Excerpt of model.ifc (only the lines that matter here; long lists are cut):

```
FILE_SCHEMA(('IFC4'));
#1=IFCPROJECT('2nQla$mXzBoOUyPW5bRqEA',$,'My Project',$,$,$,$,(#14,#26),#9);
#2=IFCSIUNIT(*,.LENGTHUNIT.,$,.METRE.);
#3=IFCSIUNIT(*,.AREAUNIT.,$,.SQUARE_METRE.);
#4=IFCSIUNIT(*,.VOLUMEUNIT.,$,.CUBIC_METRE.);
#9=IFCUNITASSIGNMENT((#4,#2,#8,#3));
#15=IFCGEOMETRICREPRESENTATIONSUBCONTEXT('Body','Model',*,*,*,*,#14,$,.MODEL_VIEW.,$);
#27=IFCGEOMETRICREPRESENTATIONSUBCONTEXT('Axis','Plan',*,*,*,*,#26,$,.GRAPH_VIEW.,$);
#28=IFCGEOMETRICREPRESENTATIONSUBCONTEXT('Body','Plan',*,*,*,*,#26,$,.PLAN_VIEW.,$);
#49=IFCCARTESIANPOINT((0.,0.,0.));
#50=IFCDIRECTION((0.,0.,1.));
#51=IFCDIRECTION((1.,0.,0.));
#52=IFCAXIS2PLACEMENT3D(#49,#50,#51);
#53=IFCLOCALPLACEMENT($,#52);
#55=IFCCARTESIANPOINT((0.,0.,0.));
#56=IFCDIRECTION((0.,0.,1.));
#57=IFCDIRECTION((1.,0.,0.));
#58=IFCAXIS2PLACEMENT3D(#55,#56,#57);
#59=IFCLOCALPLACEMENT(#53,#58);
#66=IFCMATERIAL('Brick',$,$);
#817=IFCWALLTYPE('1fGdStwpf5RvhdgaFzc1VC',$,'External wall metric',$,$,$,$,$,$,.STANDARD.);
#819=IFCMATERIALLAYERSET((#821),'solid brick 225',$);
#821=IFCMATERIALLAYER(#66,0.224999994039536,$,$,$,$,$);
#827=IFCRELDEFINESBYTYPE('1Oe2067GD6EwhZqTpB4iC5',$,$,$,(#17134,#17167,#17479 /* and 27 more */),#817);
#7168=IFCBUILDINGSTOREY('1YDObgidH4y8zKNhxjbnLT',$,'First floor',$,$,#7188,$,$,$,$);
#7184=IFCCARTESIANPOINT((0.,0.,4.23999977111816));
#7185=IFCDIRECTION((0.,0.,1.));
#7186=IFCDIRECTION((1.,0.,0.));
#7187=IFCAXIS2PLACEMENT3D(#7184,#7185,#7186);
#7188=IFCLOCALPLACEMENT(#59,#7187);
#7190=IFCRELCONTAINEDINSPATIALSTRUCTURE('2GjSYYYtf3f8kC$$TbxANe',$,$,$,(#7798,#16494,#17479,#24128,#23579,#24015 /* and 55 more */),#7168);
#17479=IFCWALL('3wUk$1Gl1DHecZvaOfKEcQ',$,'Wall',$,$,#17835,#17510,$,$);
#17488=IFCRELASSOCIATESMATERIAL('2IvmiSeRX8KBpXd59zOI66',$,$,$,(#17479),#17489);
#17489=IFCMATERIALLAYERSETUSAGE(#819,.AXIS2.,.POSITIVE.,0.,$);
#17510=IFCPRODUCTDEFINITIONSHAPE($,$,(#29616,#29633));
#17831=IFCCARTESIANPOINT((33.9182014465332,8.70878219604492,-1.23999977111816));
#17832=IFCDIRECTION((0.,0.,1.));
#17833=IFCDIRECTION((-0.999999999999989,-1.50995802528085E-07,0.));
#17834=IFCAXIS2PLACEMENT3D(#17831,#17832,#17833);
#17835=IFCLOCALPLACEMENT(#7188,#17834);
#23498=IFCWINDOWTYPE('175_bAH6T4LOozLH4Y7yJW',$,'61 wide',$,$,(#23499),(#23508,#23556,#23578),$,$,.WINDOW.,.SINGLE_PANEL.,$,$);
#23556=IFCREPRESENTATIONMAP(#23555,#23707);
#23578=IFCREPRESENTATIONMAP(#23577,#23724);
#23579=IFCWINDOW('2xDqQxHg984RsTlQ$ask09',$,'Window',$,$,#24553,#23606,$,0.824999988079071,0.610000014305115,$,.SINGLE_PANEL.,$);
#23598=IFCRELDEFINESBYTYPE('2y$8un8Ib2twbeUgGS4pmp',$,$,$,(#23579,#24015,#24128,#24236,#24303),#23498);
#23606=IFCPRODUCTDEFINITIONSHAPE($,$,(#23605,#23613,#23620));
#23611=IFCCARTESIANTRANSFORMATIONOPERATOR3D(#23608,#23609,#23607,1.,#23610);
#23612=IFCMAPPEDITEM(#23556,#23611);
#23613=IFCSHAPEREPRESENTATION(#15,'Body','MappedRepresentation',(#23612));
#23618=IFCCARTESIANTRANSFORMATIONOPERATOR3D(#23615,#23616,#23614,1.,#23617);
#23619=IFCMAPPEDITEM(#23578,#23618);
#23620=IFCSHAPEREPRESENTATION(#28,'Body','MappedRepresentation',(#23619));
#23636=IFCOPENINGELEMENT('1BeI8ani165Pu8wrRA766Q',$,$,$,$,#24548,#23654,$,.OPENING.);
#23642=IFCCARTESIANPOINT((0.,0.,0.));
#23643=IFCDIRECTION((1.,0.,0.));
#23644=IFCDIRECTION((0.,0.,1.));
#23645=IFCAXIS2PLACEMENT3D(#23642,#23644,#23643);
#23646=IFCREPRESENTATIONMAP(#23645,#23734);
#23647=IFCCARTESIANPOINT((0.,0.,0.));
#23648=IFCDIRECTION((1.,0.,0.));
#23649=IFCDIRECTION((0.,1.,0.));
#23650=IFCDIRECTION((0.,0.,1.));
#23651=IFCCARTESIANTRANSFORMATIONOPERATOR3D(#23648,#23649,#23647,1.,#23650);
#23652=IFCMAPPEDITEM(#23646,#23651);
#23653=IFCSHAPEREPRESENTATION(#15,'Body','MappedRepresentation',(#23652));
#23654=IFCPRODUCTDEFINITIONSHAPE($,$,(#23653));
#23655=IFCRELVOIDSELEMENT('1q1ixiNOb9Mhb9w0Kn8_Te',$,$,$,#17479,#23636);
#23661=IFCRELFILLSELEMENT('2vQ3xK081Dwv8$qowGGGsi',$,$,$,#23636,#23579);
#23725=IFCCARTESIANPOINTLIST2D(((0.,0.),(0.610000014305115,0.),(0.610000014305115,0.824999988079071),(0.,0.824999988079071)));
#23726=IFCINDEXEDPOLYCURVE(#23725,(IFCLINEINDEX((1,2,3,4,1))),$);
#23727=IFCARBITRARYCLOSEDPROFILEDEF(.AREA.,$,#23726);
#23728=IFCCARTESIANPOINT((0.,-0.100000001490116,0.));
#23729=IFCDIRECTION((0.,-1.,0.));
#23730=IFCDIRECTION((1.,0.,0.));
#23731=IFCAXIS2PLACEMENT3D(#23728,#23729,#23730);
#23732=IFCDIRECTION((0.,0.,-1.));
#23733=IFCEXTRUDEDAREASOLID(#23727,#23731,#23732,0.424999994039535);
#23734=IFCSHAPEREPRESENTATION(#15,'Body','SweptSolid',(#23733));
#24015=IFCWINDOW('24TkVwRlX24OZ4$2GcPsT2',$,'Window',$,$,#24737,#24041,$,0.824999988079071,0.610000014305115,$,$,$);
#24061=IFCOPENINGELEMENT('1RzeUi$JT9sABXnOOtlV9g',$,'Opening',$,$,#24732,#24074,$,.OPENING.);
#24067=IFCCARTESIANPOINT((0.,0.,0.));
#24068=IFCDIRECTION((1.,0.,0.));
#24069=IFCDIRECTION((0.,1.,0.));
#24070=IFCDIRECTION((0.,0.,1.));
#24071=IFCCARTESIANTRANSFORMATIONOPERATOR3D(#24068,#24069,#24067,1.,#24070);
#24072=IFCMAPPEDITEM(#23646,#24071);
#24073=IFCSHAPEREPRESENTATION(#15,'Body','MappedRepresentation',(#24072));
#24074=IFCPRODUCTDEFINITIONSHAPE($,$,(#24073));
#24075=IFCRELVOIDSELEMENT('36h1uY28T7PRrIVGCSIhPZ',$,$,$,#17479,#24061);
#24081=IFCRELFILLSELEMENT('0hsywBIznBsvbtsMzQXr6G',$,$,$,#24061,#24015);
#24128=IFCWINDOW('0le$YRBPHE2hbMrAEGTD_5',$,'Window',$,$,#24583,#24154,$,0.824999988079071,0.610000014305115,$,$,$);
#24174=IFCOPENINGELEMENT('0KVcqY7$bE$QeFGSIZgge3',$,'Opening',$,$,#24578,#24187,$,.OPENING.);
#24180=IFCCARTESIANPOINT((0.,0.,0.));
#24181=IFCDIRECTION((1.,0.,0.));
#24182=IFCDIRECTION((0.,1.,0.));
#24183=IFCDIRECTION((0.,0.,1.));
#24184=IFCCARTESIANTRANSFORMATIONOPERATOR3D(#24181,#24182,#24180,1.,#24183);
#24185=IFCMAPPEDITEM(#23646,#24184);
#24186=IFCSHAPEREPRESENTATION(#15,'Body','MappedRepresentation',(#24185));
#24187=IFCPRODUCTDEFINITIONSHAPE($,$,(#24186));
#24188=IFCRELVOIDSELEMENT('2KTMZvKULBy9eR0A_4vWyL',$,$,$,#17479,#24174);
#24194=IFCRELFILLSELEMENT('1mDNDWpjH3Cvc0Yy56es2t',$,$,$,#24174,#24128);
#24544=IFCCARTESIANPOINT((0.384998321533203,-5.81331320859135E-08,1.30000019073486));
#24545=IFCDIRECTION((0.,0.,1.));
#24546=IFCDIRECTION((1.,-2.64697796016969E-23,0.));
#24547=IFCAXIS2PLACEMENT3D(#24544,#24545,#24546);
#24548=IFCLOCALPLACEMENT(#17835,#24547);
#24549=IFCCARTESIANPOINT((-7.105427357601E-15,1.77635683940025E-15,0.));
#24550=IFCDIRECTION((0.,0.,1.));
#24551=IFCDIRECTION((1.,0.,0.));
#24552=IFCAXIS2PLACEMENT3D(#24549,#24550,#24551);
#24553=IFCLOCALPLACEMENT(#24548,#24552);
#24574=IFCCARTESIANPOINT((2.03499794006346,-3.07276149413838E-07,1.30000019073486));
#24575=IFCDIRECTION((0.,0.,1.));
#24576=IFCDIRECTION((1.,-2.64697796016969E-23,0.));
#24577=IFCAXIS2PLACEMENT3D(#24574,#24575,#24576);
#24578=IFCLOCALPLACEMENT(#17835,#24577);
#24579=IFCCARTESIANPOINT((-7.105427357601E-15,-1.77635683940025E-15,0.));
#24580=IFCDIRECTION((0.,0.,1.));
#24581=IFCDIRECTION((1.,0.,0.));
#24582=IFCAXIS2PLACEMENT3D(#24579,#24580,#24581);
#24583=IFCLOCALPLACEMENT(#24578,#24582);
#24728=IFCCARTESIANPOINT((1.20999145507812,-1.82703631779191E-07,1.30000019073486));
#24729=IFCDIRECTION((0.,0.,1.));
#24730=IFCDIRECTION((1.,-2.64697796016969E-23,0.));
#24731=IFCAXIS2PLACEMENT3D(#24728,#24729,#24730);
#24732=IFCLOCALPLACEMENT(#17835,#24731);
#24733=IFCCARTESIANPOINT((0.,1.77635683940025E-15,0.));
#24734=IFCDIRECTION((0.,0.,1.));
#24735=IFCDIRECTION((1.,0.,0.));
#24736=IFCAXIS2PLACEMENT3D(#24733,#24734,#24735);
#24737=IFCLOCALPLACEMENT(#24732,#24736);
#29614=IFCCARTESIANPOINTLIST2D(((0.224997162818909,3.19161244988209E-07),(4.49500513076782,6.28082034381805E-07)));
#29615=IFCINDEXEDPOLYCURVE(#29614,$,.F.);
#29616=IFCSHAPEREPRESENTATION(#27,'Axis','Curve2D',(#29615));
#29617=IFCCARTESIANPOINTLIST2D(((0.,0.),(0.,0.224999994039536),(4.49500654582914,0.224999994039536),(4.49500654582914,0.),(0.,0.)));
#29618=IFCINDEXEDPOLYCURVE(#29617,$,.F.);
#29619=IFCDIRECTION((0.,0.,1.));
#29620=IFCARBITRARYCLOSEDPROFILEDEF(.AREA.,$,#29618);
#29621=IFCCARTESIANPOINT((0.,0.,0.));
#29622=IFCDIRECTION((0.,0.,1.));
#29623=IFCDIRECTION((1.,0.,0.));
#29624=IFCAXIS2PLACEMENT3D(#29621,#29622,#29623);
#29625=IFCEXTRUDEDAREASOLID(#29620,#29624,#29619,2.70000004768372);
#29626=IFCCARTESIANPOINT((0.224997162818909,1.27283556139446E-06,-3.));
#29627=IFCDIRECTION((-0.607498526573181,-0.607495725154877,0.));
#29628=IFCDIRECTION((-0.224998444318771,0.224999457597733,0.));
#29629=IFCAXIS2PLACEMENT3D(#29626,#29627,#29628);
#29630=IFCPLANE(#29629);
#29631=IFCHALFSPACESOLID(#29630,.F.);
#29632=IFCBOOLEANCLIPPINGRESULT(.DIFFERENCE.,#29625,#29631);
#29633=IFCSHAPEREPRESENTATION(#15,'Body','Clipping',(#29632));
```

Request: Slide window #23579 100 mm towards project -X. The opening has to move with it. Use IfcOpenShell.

```python
import ifcopenshell
import ifcopenshell.api.geometry
import ifcopenshell.util.placement

model = ifcopenshell.open("model.ifc")

window = model.by_guid("2xDqQxHg984RsTlQ$ask09")
opening = window.FillsVoids[0].RelatingOpeningElement
wall = opening.VoidsElements[0].RelatingBuildingElement

wall_matrix = ifcopenshell.util.placement.get_local_placement(wall.ObjectPlacement)
shift = wall_matrix[:3, 0] * 0.1
before = ifcopenshell.util.placement.get_local_placement(window.ObjectPlacement)[:3, 3].copy()

# The window is placed relative to its opening, so it follows when the opening moves.
matrix = ifcopenshell.util.placement.get_local_placement(opening.ObjectPlacement)
matrix[:3, 3] += shift
ifcopenshell.api.geometry.edit_object_placement(
    model, product=opening, matrix=matrix, is_si=False, should_transform_children=True
)

after = ifcopenshell.util.placement.get_local_placement(window.ObjectPlacement)[:3, 3]
print("window moved by", (after - before).round(3) + 0.0)

model.write("model_edited.ifc")
```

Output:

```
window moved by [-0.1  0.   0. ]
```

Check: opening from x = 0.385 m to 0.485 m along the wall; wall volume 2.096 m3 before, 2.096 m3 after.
